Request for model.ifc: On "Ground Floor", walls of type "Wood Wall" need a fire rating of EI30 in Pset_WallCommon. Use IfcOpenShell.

First a look at what the model holds.

```python
import ifcopenshell
import ifcopenshell.util.element

model = ifcopenshell.open("model.ifc")
print(model.schema)
storey = next(s for s in model.by_type("IfcBuildingStorey") if s.Name == "Ground Floor")
walls = [e for e in ifcopenshell.util.element.get_decomposition(storey) if e.is_a("IfcWall")]
seen = {}
for e in walls:
    element_type = ifcopenshell.util.element.get_type(e)
    key = (element_type.Name if element_type != e and element_type else None, ifcopenshell.util.element.get_pset(e, "Pset_WallCommon", "FireRating"))
    seen[key] = seen.get(key, 0) + 1
for (name, value), count in sorted(seen.items(), key=str):
    print(count, "x", name, "|", value)
```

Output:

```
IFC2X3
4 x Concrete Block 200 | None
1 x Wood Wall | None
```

```python
import ifcopenshell
import ifcopenshell.api.pset
import ifcopenshell.util.element

model = ifcopenshell.open("model.ifc")

storey = next(s for s in model.by_type("IfcBuildingStorey") if s.Name == "Ground Floor")
walls = [e for e in ifcopenshell.util.element.get_decomposition(storey) if e.is_a("IfcWall")]

count = 0
for e in walls:
    element_type = ifcopenshell.util.element.get_type(e)
    if element_type in (None, e) or element_type.Name != "Wood Wall":
        continue
    # add_pset returns the element's existing set when there is one.
    pset = ifcopenshell.api.pset.add_pset(model, product=e, name="Pset_WallCommon")
    ifcopenshell.api.pset.edit_pset(model, pset=pset, properties={"FireRating": "EI30"})
    count += 1

print(count, "walls updated")

model.write("model_edited.ifc")
```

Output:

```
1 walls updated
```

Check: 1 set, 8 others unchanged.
